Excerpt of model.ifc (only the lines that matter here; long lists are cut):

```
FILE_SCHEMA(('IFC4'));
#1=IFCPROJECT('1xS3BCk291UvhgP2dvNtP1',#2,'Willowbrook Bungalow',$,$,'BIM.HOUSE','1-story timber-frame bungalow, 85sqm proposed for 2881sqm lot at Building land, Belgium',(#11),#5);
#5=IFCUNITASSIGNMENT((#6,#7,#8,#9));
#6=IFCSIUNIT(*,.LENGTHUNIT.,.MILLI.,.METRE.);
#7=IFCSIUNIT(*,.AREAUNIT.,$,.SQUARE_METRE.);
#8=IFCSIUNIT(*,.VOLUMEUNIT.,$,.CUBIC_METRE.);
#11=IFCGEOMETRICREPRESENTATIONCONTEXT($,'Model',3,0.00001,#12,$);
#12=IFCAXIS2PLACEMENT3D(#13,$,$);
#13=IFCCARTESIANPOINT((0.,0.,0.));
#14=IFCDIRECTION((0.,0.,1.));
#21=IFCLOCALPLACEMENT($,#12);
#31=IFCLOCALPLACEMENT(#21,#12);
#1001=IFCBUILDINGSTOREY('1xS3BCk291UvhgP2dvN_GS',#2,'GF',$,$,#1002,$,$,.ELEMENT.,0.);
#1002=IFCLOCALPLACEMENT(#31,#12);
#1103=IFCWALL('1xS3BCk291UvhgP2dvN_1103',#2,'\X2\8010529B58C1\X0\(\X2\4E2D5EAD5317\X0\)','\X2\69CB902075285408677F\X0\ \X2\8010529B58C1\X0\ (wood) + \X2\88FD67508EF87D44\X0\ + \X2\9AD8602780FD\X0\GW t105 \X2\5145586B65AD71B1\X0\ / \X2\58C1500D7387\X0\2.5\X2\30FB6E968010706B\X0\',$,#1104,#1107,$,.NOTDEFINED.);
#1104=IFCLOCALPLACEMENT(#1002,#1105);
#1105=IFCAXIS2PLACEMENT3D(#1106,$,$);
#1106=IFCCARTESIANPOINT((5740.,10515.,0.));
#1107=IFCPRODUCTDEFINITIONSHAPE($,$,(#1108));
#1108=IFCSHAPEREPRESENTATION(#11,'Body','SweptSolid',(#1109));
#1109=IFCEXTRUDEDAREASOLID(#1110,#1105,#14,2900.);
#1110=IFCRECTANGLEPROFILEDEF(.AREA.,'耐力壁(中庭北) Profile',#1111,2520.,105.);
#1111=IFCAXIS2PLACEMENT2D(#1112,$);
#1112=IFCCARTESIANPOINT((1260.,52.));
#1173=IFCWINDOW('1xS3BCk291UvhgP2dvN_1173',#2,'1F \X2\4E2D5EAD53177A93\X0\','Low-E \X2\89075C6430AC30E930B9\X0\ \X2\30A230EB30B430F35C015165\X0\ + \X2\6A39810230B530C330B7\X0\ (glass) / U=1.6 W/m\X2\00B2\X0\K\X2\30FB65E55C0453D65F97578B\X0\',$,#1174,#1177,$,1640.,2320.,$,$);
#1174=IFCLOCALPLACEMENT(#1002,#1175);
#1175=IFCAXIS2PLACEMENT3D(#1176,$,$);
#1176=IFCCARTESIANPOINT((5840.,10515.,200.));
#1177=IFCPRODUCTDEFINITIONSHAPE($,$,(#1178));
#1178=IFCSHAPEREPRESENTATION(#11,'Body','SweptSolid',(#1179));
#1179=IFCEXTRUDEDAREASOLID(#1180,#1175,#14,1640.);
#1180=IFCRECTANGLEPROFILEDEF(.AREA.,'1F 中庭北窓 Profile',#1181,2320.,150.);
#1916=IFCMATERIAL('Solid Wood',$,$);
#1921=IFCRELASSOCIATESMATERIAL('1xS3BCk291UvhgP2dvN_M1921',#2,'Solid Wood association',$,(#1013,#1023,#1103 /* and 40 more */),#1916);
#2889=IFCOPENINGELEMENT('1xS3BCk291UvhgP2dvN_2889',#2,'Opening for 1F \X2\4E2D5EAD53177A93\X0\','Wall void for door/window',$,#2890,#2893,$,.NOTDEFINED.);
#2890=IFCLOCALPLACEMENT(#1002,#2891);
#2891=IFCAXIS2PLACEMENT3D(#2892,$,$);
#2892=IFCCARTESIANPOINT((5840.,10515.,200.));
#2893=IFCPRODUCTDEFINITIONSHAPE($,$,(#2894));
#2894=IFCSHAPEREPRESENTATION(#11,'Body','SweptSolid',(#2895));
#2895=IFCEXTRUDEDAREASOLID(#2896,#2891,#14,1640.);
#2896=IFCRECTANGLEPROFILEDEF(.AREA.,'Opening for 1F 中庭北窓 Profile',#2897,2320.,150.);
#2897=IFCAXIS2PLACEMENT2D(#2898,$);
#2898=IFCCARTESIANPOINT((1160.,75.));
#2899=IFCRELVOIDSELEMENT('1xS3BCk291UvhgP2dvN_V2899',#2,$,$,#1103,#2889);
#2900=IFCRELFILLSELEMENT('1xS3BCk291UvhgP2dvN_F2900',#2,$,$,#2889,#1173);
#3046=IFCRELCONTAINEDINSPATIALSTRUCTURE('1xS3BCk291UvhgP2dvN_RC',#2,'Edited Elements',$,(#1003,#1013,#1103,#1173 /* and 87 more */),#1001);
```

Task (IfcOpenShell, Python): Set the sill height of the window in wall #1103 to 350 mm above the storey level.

```python
import numpy as np
import ifcopenshell
import ifcopenshell.api.geometry
import ifcopenshell.geom
import ifcopenshell.util.element
import ifcopenshell.util.placement
import ifcopenshell.util.shape
import ifcopenshell.util.unit

model = ifcopenshell.open("model.ifc")
unit_scale = ifcopenshell.util.unit.calculate_unit_scale(model)

window = model.by_guid("1xS3BCk291UvhgP2dvN_1173")
opening = window.FillsVoids[0].RelatingOpeningElement
storey = ifcopenshell.util.element.get_container(window, ifc_class="IfcBuildingStorey")
level = ifcopenshell.util.placement.get_local_placement(storey.ObjectPlacement)[2, 3]

# The opening's origin need not be at the sill, so measure its lowest point.
shape = ifcopenshell.geom.create_shape(ifcopenshell.geom.settings(), opening)
bottom = ifcopenshell.util.shape.get_shape_bottom_elevation(shape, shape.geometry) / unit_scale
dz = level + 350.0 - bottom

shift = np.array([0.0, 0.0, dz])
# The window is not placed relative to its opening, so move both.
for product in (opening, window):
    matrix = ifcopenshell.util.placement.get_local_placement(product.ObjectPlacement)
    matrix[:3, 3] += shift
    ifcopenshell.api.geometry.edit_object_placement(model, product=product, matrix=matrix, is_si=False)

print(f"moved by {dz * unit_scale:+.3f} m")

model.write("model_v2.ifc")
```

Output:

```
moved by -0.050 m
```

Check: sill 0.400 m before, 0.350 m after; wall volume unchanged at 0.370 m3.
